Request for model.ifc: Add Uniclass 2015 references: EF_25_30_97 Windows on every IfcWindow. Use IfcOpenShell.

First a look at what the model holds.

```python
import ifcopenshell

model = ifcopenshell.open("model.ifc")
print(model.schema)
print("classifications:", [c.Name for c in model.by_type("IfcClassification")])
for ifc_class in ("IfcDoor", "IfcRoof", "IfcStair", "IfcWall", "IfcWindow"):
    print(ifc_class, len(model.by_type(ifc_class)))
```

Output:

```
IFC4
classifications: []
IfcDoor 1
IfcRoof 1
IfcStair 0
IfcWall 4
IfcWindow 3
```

```python
import ifcopenshell
import ifcopenshell.api.classification

model = ifcopenshell.open("model.ifc")

system = ifcopenshell.api.classification.add_classification(model, classification="Uniclass 2015")

codes = {
    "IfcWindow": ("EF_25_30_97", "Windows"),
}
for ifc_class, (code, name) in codes.items():
    products = model.by_type(ifc_class)
    ifcopenshell.api.classification.add_reference(
        model, products=products, classification=system, identification=code, name=name
    )
    print(code, len(products))

model.write("model_rev.ifc")
```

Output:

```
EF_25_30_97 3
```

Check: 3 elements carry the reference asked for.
